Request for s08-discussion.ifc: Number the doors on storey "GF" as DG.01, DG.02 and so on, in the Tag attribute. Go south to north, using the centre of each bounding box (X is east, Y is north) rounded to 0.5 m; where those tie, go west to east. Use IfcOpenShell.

First a look at what the model holds.

```python
import ifcopenshell
import ifcopenshell.util.element
import ifcopenshell.util.placement

model = ifcopenshell.open("s08-discussion.ifc")
print(model.schema)
storey = next(s for s in model.by_type("IfcBuildingStorey") if s.Name == "GF")
doors = [e for e in ifcopenshell.util.element.get_decomposition(storey) if e.is_a("IfcDoor")]
for e in sorted(doors, key=lambda e: e.id()):
    origin = ifcopenshell.util.placement.get_local_placement(e.ObjectPlacement)[:3, 3]
    print(e.id(), e.Tag, e.Name, origin.round(2) + 0.0, sep=" | ")
```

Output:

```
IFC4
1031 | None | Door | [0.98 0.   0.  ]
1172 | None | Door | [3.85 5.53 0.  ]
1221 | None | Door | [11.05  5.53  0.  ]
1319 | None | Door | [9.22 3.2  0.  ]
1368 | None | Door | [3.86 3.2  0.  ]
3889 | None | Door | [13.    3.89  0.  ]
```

```python
import ifcopenshell
import ifcopenshell.geom
import ifcopenshell.util.element
import ifcopenshell.util.shape

model = ifcopenshell.open("s08-discussion.ifc")
settings = ifcopenshell.geom.settings()
settings.set("use-world-coords", True)


def centre(element):
    shape = ifcopenshell.geom.create_shape(settings, element)
    return ifcopenshell.util.shape.get_bbox_centroid(shape.geometry)


storey = next(s for s in model.by_type("IfcBuildingStorey") if s.Name == "GF")
doors = [e for e in ifcopenshell.util.element.get_decomposition(storey) if e.is_a("IfcDoor")]

# Insertion points can sit at a corner or the storey origin, so sort by the geometry (in metres).
centres = {e: centre(e) for e in doors}
doors.sort(key=lambda e: (round(centres[e][1] / 0.5), centres[e][0]))

for i, e in enumerate(doors, start=1):
    number = f"DG.{i:02d}"
    e.Tag = number
    print(e.id(), number)

model.write("s08-discussion_rev.ifc")
```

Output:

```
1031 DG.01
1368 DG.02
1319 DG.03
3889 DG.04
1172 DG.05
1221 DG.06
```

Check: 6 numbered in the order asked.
